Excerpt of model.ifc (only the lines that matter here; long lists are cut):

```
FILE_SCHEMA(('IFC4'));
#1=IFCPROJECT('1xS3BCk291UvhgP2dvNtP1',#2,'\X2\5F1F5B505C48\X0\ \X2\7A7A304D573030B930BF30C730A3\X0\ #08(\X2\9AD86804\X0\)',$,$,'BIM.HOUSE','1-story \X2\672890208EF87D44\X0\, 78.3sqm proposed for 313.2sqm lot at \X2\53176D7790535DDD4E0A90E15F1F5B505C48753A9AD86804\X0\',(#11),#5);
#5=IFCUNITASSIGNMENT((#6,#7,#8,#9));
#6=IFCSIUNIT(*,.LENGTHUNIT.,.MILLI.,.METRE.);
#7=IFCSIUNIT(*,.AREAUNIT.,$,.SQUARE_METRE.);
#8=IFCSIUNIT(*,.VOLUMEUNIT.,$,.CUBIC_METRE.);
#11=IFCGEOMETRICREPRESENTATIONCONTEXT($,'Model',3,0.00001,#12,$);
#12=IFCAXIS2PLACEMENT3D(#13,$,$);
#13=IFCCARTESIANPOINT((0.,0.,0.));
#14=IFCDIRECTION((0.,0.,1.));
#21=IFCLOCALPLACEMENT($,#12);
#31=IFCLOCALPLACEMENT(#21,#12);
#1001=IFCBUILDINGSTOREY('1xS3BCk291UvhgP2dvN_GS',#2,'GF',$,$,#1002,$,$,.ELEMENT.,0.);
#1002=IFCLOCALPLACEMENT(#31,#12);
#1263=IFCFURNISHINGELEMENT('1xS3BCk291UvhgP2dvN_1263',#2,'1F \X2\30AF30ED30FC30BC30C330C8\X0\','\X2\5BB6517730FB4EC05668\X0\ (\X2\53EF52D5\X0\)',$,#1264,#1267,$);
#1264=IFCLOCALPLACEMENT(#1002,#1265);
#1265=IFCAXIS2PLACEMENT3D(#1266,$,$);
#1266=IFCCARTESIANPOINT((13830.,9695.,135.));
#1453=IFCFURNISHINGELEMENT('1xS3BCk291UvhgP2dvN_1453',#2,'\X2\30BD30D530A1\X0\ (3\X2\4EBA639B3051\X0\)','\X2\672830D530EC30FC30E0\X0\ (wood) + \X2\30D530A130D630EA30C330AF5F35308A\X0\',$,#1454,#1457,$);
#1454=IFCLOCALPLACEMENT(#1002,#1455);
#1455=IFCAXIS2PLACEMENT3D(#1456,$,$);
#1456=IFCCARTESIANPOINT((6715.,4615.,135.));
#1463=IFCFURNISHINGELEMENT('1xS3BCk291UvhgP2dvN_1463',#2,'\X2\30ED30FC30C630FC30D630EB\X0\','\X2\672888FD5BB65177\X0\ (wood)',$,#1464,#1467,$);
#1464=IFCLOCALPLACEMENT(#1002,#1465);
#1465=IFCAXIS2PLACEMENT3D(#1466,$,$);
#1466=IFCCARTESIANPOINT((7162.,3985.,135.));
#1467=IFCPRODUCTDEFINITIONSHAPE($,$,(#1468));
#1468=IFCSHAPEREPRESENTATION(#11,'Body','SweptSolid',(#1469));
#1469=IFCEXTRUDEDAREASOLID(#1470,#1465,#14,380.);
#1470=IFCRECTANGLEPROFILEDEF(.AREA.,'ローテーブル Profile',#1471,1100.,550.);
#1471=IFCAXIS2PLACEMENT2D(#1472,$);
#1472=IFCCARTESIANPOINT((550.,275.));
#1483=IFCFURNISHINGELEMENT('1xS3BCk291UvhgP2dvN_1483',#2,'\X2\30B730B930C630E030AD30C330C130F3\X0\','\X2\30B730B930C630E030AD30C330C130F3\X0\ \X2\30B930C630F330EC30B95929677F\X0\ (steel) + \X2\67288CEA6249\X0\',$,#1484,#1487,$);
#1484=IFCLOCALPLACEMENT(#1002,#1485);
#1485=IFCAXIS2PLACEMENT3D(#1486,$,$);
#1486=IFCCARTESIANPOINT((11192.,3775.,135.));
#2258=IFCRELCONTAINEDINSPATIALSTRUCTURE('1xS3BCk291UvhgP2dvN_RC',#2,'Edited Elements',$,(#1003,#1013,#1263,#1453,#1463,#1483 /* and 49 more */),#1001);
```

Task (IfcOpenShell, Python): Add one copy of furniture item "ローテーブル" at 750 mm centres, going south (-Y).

```python
import numpy as np
import ifcopenshell
import ifcopenshell.api.geometry
import ifcopenshell.api.root
import ifcopenshell.util.element
import ifcopenshell.util.placement
import ifcopenshell.util.unit

model = ifcopenshell.open("model.ifc")
unit_scale = ifcopenshell.util.unit.calculate_unit_scale(model)


def reuse_history(source, copy):
    """copy_class also copies each property set's owner history, people and application; keep the originals."""
    for rel in copy.IsDefinedBy:
        if rel.is_a("IfcRelDefinesByProperties") and (history := rel.RelatingPropertyDefinition.OwnerHistory):
            rel.RelatingPropertyDefinition.OwnerHistory = source.OwnerHistory
            ifcopenshell.util.element.remove_deep2(model, history)


source = model.by_guid("1xS3BCk291UvhgP2dvN_1463")
base = ifcopenshell.util.placement.get_local_placement(source.ObjectPlacement)
step = np.array([0.0, -1.0, 0.0]) * 0.75 / unit_scale

for i in range(1, 2):
    copy = ifcopenshell.api.root.copy_class(model, product=source)
    copy.Representation = ifcopenshell.util.element.copy_deep(
        model, source.Representation, exclude=["IfcGeometricRepresentationContext", "IfcRepresentationMap"]
    )
    reuse_history(source, copy)
    matrix = base.copy()
    matrix[:3, 3] += i * step
    print("added at", matrix[:3, 3].round(3) + 0.0)
    ifcopenshell.api.geometry.edit_object_placement(model, product=copy, matrix=matrix, is_si=False)

model.write("model-out.ifc")
```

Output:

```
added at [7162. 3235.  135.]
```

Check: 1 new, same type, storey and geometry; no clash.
